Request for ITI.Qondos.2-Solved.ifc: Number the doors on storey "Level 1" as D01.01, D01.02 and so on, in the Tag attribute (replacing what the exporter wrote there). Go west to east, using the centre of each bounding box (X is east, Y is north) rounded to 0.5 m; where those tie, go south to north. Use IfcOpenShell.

First a look at what the model holds.

```python
import ifcopenshell
import ifcopenshell.util.element
import ifcopenshell.util.placement

model = ifcopenshell.open("ITI.Qondos.2-Solved.ifc")
print(model.schema)
storey = next(s for s in model.by_type("IfcBuildingStorey") if s.Name == "Level 1")
doors = [e for e in ifcopenshell.util.element.get_decomposition(storey) if e.is_a("IfcDoor")]
for e in sorted(doors, key=lambda e: e.id()):
    origin = ifcopenshell.util.placement.get_local_placement(e.ObjectPlacement)[:3, 3]
    print(e.id(), e.Tag, e.Name, origin.round(2) + 0.0, sep=" | ")
```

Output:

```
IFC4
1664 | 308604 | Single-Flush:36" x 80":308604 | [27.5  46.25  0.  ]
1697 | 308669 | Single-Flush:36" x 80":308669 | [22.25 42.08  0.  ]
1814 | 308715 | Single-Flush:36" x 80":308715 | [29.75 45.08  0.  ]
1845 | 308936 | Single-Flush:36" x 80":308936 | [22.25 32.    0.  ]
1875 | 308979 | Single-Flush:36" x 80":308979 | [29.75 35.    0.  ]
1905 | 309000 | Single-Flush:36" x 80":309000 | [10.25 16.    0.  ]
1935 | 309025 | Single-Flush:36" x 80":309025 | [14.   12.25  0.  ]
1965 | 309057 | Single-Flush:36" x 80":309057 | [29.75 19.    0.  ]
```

```python
import ifcopenshell
import ifcopenshell.geom
import ifcopenshell.util.element
import ifcopenshell.util.shape

model = ifcopenshell.open("ITI.Qondos.2-Solved.ifc")
settings = ifcopenshell.geom.settings()
settings.set("use-world-coords", True)


def centre(element):
    shape = ifcopenshell.geom.create_shape(settings, element)
    return ifcopenshell.util.shape.get_bbox_centroid(shape.geometry)


storey = next(s for s in model.by_type("IfcBuildingStorey") if s.Name == "Level 1")
doors = [e for e in ifcopenshell.util.element.get_decomposition(storey) if e.is_a("IfcDoor")]

# Insertion points can sit at a corner or the storey origin, so sort by the geometry (in metres).
centres = {e: centre(e) for e in doors}
doors.sort(key=lambda e: (round(centres[e][0] / 0.5), centres[e][1]))

for i, e in enumerate(doors, start=1):
    number = f"D01.{i:02d}"
    e.Tag = number
    print(e.id(), number)

model.write("ITI.Qondos.2-Solved_rev.ifc")
```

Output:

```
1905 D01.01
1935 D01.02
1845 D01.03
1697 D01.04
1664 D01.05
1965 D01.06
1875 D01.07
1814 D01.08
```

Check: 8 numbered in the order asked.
